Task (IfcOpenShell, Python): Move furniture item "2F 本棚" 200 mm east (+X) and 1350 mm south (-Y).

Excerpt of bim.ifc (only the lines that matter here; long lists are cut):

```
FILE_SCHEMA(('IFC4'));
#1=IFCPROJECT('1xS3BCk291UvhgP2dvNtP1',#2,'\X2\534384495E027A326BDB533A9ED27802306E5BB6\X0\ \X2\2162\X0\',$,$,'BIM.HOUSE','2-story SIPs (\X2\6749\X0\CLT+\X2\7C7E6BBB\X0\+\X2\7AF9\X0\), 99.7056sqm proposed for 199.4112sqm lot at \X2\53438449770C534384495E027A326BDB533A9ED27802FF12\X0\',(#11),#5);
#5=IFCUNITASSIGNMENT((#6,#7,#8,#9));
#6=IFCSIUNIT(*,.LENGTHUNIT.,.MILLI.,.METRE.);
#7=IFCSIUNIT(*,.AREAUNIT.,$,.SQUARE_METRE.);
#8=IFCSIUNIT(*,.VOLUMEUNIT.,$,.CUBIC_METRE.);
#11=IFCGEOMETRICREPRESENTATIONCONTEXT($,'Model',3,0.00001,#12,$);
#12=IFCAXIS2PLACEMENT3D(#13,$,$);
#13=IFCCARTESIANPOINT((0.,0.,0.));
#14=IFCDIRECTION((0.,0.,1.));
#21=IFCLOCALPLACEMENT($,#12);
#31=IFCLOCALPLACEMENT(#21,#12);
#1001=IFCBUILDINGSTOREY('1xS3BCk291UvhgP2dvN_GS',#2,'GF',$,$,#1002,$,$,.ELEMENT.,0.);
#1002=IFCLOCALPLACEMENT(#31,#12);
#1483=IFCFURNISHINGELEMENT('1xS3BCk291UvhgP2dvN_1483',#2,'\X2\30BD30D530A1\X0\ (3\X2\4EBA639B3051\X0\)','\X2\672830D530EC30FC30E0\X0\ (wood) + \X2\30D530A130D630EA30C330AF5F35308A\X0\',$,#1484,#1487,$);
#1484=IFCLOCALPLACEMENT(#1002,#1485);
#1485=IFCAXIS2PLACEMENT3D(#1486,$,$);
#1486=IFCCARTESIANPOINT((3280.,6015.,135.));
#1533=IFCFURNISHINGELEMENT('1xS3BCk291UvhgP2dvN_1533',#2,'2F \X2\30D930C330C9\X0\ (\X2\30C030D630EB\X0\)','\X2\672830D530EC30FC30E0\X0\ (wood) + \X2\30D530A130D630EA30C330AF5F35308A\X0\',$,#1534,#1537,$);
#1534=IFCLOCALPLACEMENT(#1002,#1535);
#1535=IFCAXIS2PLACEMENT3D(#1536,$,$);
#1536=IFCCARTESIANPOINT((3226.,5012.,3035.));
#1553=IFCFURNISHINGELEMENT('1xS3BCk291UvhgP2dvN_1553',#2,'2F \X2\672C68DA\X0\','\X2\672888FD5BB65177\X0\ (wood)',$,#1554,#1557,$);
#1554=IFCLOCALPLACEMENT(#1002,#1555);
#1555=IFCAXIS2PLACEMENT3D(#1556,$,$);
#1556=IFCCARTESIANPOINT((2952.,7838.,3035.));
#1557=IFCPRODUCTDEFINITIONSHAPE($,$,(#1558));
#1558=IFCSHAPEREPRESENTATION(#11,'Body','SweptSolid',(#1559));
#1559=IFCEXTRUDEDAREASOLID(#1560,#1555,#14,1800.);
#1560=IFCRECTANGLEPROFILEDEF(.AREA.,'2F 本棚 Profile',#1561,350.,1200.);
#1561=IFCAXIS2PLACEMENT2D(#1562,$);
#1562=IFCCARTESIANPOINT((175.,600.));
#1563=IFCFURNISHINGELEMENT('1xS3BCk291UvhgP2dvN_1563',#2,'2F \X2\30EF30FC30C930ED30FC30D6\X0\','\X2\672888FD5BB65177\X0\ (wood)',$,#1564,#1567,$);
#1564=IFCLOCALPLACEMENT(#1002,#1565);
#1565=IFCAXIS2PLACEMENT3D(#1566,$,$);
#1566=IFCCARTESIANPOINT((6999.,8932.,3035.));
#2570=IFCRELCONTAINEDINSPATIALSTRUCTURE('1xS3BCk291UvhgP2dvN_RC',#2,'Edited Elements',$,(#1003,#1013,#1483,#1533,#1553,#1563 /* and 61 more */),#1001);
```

```python
import ifcopenshell
import ifcopenshell.api.geometry
import ifcopenshell.util.placement

model = ifcopenshell.open("bim.ifc")

item = model.by_guid("1xS3BCk291UvhgP2dvN_1553")
matrix = ifcopenshell.util.placement.get_local_placement(item.ObjectPlacement)
matrix[0, 3] += 200.0
matrix[1, 3] -= 1350.0
ifcopenshell.api.geometry.edit_object_placement(model, product=item, matrix=matrix, is_si=False)

print(ifcopenshell.util.placement.get_local_placement(item.ObjectPlacement).round(3) + 0.0)

model.write("bim_updated.ifc")
```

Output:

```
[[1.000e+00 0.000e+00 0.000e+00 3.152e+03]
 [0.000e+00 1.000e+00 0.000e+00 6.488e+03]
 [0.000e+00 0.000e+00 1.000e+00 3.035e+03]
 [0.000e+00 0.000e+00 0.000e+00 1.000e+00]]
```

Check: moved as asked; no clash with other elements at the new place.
